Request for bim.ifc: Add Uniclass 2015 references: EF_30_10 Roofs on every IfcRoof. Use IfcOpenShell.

First a look at what the model holds.

```python
import ifcopenshell

model = ifcopenshell.open("bim.ifc")
print(model.schema)
print("classifications:", [c.Name for c in model.by_type("IfcClassification")])
for ifc_class in ("IfcDoor", "IfcRoof", "IfcStair", "IfcWall", "IfcWindow"):
    print(ifc_class, len(model.by_type(ifc_class)))
```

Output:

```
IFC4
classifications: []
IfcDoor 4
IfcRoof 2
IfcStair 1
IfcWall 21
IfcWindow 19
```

```python
import ifcopenshell
import ifcopenshell.api.classification

model = ifcopenshell.open("bim.ifc")

system = ifcopenshell.api.classification.add_classification(model, classification="Uniclass 2015")

codes = {
    "IfcRoof": ("EF_30_10", "Roofs"),
}
for ifc_class, (code, name) in codes.items():
    products = model.by_type(ifc_class)
    ifcopenshell.api.classification.add_reference(
        model, products=products, classification=system, identification=code, name=name
    )
    print(code, len(products))

model.write("bim_rev.ifc")
```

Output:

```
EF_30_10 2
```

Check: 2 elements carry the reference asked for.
